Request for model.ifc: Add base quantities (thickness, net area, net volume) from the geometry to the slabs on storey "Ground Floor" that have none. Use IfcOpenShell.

First a look at what the model holds.

```python
import ifcopenshell
import ifcopenshell.util.element
import ifcopenshell.util.unit

model = ifcopenshell.open("model.ifc")
print(model.schema)
for unit_type in ("LENGTHUNIT", "AREAUNIT", "VOLUMEUNIT"):
    print(unit_type, ifcopenshell.util.unit.calculate_unit_scale(model, unit_type))
storey = next(s for s in model.by_type("IfcBuildingStorey") if s.Name == "Ground Floor")
slabs = [e for e in ifcopenshell.util.element.get_decomposition(storey) if e.is_a("IfcSlab")]
for e in sorted(slabs, key=lambda e: e.id()):
    print(e.id(), e.is_a(), e.Name, list(ifcopenshell.util.element.get_psets(e, qtos_only=True)), sep=" | ")
```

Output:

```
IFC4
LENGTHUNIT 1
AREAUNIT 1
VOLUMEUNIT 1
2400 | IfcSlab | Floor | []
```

```python
import ifcopenshell
import ifcopenshell.api.pset
import ifcopenshell.geom
import ifcopenshell.util.element
import ifcopenshell.util.shape
import ifcopenshell.util.unit

model = ifcopenshell.open("model.ifc")
unit_scale = ifcopenshell.util.unit.calculate_unit_scale(model)
area_scale = ifcopenshell.util.unit.calculate_unit_scale(model, "AREAUNIT")
volume_scale = ifcopenshell.util.unit.calculate_unit_scale(model, "VOLUMEUNIT")
settings = ifcopenshell.geom.settings()

storey = next(s for s in model.by_type("IfcBuildingStorey") if s.Name == "Ground Floor")
slabs = [e for e in ifcopenshell.util.element.get_decomposition(storey) if e.is_a("IfcSlab")]

for e in sorted(slabs, key=lambda e: e.id()):
    if ifcopenshell.util.element.get_psets(e, qtos_only=True, should_inherit=False):
        continue
    # Geometry comes back in metres, in the element's own axes.
    shape = ifcopenshell.geom.create_shape(settings, e)
    values = {
        "Width": ifcopenshell.util.shape.get_z(shape.geometry) / unit_scale,
        "NetArea": ifcopenshell.util.shape.get_footprint_area(shape.geometry) / area_scale,
        "NetVolume": ifcopenshell.util.shape.get_volume(shape.geometry) / volume_scale,
    }
    qto = ifcopenshell.api.pset.add_qto(model, product=e, name="Qto_SlabBaseQuantities")
    ifcopenshell.api.pset.edit_qto(model, qto=qto, properties=values)
    print(e.id(), {k: round(v, 3) for k, v in values.items()})

model.write("model_rev.ifc")
```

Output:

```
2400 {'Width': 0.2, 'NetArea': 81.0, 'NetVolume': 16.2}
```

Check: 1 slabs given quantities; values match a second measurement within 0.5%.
